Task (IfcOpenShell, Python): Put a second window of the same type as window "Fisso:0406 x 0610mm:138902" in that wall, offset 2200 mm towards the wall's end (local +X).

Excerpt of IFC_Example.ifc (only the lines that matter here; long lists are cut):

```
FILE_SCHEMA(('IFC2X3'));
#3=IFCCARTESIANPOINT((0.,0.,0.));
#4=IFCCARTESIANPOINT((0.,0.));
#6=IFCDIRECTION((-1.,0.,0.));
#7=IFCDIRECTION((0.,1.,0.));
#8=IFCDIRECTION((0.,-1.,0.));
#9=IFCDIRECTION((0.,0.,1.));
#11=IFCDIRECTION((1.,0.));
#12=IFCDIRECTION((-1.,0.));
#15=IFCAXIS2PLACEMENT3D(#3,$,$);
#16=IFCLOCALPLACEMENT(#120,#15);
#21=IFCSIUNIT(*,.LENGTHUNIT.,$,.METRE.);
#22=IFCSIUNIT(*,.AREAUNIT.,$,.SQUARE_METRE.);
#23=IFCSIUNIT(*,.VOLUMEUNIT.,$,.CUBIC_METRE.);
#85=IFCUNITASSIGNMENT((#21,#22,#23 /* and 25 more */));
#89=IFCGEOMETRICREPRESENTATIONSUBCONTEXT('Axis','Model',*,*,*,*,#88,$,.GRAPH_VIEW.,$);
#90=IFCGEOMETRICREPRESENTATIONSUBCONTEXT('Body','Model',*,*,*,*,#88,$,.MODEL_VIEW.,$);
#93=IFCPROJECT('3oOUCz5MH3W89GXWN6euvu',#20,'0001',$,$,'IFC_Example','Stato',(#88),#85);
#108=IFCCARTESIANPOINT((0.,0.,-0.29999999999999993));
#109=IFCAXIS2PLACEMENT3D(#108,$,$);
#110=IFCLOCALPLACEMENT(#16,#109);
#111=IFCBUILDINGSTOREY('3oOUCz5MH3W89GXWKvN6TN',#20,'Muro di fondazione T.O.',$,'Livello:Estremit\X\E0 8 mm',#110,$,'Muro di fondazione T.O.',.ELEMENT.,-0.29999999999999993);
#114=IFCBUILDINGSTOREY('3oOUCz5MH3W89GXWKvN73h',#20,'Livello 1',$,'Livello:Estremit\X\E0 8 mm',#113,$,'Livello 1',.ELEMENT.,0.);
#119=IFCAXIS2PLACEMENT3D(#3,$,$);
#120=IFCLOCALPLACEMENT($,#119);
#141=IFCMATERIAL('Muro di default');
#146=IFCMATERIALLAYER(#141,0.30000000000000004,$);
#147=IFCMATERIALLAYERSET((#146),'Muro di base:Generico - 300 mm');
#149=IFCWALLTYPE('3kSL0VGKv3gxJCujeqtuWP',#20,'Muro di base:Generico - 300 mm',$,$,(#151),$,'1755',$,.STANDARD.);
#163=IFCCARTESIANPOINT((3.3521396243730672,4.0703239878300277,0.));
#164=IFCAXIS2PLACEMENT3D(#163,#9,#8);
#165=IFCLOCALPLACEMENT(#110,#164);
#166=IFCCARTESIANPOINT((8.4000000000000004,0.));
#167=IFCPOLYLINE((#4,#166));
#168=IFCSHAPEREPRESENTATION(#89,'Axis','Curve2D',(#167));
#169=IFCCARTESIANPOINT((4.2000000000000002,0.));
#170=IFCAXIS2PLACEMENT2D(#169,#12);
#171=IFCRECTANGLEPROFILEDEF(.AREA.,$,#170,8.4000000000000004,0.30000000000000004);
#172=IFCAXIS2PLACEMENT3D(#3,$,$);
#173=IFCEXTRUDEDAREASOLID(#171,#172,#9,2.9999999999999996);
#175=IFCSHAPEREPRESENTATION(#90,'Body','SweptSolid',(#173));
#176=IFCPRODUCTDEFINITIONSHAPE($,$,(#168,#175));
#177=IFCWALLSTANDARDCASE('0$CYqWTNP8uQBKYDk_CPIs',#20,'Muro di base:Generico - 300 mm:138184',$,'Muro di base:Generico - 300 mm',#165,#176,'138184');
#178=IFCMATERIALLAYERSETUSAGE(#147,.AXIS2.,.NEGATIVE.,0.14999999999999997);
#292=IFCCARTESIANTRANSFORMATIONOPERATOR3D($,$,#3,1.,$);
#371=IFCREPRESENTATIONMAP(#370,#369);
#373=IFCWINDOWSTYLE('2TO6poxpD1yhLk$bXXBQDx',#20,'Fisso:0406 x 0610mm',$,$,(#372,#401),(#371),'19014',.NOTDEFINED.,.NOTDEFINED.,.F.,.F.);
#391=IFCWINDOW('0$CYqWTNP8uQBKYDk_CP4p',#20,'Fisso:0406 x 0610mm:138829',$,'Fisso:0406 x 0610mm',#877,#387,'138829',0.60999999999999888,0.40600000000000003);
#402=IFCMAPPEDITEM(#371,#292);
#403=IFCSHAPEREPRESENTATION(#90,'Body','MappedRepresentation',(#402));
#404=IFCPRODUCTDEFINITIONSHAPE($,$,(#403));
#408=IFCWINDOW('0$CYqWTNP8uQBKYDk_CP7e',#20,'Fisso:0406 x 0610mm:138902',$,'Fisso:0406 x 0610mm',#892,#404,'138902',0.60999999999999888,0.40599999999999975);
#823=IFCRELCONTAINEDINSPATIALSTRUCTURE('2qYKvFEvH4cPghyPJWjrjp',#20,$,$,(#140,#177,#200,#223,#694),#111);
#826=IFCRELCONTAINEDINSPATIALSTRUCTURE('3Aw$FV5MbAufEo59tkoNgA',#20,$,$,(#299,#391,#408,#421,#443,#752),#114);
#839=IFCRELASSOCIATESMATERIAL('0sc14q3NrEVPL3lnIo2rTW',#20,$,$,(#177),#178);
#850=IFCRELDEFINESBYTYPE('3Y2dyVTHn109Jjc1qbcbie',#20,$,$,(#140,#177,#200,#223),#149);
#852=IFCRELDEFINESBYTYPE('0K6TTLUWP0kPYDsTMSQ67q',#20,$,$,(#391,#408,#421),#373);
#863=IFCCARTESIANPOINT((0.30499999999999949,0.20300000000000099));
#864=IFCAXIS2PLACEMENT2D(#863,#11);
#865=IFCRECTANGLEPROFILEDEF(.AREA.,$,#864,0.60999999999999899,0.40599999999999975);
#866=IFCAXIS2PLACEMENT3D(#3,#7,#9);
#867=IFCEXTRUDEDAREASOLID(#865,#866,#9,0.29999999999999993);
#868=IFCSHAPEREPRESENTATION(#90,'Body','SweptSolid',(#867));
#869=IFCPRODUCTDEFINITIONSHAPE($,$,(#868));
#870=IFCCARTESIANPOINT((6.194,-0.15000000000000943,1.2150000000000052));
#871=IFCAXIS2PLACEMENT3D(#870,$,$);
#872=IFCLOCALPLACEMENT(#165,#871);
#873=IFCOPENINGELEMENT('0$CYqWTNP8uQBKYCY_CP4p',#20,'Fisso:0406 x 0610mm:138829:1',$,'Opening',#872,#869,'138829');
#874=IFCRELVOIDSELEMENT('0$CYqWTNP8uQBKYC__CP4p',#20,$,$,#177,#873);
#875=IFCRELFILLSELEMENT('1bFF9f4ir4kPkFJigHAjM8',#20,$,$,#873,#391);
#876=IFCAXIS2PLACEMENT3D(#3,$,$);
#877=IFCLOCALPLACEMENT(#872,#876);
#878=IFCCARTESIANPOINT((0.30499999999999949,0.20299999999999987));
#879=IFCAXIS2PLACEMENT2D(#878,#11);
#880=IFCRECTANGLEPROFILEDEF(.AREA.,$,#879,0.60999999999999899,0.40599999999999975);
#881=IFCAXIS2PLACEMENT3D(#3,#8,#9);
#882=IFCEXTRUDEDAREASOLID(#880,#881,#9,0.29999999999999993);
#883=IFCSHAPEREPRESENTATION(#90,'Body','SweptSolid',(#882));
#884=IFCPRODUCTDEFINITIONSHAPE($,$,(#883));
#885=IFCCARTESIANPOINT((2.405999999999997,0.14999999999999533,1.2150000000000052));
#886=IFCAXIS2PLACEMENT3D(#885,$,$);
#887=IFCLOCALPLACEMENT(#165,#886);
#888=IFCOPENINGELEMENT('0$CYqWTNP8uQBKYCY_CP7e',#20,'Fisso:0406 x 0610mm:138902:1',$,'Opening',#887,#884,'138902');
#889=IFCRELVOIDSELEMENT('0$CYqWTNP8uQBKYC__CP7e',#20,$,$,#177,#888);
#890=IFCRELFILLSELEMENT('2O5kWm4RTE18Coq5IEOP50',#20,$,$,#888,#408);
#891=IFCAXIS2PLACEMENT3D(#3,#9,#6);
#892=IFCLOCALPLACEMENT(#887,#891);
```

```python
import ifcopenshell
import ifcopenshell.api.feature
import ifcopenshell.api.geometry
import ifcopenshell.api.root
import ifcopenshell.geom
import ifcopenshell.util.element
import ifcopenshell.util.placement
import ifcopenshell.util.shape

model = ifcopenshell.open("IFC_Example.ifc")
settings = ifcopenshell.geom.settings()


def volume(element):
    """Net volume in cubic metres, openings subtracted."""
    shape = ifcopenshell.geom.create_shape(settings, element)
    return ifcopenshell.util.shape.get_volume(shape.geometry)


def reuse_history(source, copy):
    """copy_class also copies each property set's owner history, people and application; keep the originals."""
    for rel in copy.IsDefinedBy:
        if rel.is_a("IfcRelDefinesByProperties") and (history := rel.RelatingPropertyDefinition.OwnerHistory):
            rel.RelatingPropertyDefinition.OwnerHistory = source.OwnerHistory
            ifcopenshell.util.element.remove_deep2(model, history)


window = model.by_guid("0$CYqWTNP8uQBKYDk_CP7e")
opening = window.FillsVoids[0].RelatingOpeningElement
wall = opening.VoidsElements[0].RelatingBuildingElement
before = volume(wall)
shift = ifcopenshell.util.placement.get_local_placement(wall.ObjectPlacement)[:3, 0] * 2.2

# copy_class copies the void relationship, type, container and properties, but no geometry.
new_opening = ifcopenshell.api.root.copy_class(model, product=opening)
new_opening.Representation = ifcopenshell.util.element.copy_deep(
    model, opening.Representation, exclude=["IfcGeometricRepresentationContext", "IfcRepresentationMap"]
)
new_opening.Name = "Fisso:0406 x 0610mm"
new_opening.Tag = None
new_window = ifcopenshell.api.root.copy_class(model, product=window)
new_window.Representation = ifcopenshell.util.element.copy_deep(
    model, window.Representation, exclude=["IfcGeometricRepresentationContext", "IfcRepresentationMap"]
)
new_window.Name = "Fisso:0406 x 0610mm"
new_window.Tag = None
reuse_history(window, new_window)
fills = ifcopenshell.api.feature.add_filling(model, opening=new_opening, element=new_window)
fills.OwnerHistory = new_window.OwnerHistory  # required in IFC2X3

for old, new in ((opening, new_opening), (window, new_window)):
    matrix = ifcopenshell.util.placement.get_local_placement(old.ObjectPlacement)
    matrix[:3, 3] += shift
    ifcopenshell.api.geometry.edit_object_placement(model, product=new, matrix=matrix, is_si=False)

after = volume(wall)

print(f"wall volume {before:.3f} -> {after:.3f} m3")

model.write("IFC_Example-out.ifc")
```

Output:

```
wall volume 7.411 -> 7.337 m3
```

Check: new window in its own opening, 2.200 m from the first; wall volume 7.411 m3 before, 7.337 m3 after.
